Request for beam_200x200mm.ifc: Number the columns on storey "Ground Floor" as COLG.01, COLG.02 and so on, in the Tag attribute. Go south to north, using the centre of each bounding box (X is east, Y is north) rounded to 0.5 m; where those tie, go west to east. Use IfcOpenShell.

First a look at what the model holds.

```python
import ifcopenshell
import ifcopenshell.util.element
import ifcopenshell.util.placement

model = ifcopenshell.open("beam_200x200mm.ifc")
print(model.schema)
storey = next(s for s in model.by_type("IfcBuildingStorey") if s.Name == "Ground Floor")
columns = [e for e in ifcopenshell.util.element.get_decomposition(storey) if e.is_a("IfcColumn")]
for e in sorted(columns, key=lambda e: e.id()):
    origin = ifcopenshell.util.placement.get_local_placement(e.ObjectPlacement)[:3, 3]
    print(e.id(), e.Tag, e.Name, origin.round(2) + 0.0, sep=" | ")
```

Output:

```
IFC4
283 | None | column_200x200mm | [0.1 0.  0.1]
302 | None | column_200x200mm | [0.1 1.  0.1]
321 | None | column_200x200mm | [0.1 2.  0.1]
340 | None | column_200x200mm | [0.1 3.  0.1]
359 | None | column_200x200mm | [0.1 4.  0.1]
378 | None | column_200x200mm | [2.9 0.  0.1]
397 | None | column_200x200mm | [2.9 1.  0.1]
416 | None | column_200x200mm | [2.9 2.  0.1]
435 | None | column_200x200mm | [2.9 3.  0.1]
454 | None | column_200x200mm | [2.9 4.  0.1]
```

```python
import ifcopenshell
import ifcopenshell.geom
import ifcopenshell.util.element
import ifcopenshell.util.shape

model = ifcopenshell.open("beam_200x200mm.ifc")
settings = ifcopenshell.geom.settings()
settings.set("use-world-coords", True)


def centre(element):
    shape = ifcopenshell.geom.create_shape(settings, element)
    return ifcopenshell.util.shape.get_bbox_centroid(shape.geometry)


storey = next(s for s in model.by_type("IfcBuildingStorey") if s.Name == "Ground Floor")
columns = [e for e in ifcopenshell.util.element.get_decomposition(storey) if e.is_a("IfcColumn")]

# Insertion points can sit at a corner or the storey origin, so sort by the geometry (in metres).
centres = {e: centre(e) for e in columns}
columns.sort(key=lambda e: (round(centres[e][1] / 0.5), centres[e][0]))

for i, e in enumerate(columns, start=1):
    number = f"COLG.{i:02d}"
    e.Tag = number
    print(e.id(), number)

model.write("beam_200x200mm_edited.ifc")
```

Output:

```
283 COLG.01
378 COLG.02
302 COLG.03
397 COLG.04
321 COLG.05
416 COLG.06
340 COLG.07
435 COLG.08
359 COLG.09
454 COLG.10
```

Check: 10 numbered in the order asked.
